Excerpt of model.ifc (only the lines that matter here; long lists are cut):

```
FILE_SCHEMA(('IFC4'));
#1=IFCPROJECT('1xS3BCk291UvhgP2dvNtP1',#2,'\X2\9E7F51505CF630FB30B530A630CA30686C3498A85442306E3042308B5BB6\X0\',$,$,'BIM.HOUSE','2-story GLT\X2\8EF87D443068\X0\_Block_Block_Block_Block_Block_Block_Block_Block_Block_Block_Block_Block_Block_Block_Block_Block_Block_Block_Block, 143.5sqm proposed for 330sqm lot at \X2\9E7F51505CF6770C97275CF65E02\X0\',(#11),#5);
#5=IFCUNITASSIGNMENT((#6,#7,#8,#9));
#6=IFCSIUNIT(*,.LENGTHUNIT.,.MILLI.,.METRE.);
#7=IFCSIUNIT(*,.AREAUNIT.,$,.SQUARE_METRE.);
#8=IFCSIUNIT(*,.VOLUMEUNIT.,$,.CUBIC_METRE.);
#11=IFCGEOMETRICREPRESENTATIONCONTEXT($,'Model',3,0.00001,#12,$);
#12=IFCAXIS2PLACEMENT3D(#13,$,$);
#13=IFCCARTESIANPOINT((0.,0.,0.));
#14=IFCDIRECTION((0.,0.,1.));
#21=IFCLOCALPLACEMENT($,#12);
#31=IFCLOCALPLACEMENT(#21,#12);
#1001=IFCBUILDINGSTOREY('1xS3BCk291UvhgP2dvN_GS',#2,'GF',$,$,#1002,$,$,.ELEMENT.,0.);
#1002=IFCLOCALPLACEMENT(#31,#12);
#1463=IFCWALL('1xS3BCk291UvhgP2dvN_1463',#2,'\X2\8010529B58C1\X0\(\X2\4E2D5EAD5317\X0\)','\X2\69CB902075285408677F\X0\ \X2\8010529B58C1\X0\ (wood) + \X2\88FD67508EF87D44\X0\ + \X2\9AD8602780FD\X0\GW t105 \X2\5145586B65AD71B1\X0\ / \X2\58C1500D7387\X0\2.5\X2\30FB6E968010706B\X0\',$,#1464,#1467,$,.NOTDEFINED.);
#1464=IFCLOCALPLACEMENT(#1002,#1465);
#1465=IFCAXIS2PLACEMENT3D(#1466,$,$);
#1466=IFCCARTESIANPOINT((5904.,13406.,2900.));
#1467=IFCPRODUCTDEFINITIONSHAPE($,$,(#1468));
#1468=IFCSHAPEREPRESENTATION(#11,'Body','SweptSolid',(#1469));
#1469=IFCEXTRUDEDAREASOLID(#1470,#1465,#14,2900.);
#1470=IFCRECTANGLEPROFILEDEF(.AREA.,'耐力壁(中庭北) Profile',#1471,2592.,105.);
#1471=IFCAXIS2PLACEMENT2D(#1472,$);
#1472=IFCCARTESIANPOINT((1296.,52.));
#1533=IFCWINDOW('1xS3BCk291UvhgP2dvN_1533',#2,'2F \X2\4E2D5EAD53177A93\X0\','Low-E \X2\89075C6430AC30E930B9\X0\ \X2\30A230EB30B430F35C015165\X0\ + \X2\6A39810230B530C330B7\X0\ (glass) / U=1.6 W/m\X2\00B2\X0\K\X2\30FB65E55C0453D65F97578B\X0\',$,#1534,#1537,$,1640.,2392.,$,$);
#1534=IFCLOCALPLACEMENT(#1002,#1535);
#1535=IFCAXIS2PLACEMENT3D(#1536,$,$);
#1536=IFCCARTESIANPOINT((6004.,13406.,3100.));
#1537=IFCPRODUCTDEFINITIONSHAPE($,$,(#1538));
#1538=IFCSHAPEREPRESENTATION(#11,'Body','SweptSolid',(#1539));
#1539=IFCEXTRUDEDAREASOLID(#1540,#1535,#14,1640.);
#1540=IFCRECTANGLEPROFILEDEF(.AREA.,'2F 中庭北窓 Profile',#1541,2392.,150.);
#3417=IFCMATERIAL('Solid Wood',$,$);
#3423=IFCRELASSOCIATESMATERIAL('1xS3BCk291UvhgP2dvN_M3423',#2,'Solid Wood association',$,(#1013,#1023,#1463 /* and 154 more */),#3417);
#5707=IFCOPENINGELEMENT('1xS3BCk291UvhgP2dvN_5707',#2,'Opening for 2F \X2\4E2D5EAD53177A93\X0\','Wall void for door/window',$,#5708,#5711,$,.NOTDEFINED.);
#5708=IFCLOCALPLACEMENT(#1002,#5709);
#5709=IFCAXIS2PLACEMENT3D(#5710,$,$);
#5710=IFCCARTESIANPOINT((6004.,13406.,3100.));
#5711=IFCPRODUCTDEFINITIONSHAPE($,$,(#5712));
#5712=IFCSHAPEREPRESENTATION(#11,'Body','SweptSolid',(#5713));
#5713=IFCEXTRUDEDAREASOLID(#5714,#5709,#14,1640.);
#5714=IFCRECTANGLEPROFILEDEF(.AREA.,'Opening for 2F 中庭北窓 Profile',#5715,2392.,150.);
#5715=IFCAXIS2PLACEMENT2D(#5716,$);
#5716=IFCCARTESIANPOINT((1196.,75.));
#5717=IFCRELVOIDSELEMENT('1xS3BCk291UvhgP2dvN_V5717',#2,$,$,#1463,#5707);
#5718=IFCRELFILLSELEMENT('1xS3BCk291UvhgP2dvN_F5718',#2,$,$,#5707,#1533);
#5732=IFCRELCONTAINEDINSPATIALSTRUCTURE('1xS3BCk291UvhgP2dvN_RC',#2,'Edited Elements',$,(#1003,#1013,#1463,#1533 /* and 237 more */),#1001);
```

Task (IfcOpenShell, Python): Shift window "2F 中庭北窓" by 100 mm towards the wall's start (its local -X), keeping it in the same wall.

```python
import ifcopenshell
import ifcopenshell.api.geometry
import ifcopenshell.util.placement
import ifcopenshell.util.unit

model = ifcopenshell.open("model.ifc")
unit_scale = ifcopenshell.util.unit.calculate_unit_scale(model)

window = model.by_id(1533)
opening = window.FillsVoids[0].RelatingOpeningElement
wall = opening.VoidsElements[0].RelatingBuildingElement

wall_matrix = ifcopenshell.util.placement.get_local_placement(wall.ObjectPlacement)
shift = wall_matrix[:3, 0] * -0.1 / unit_scale
before = ifcopenshell.util.placement.get_local_placement(window.ObjectPlacement)[:3, 3].copy()

# The window is not placed relative to its opening, so move both.
for product in (opening, window):
    matrix = ifcopenshell.util.placement.get_local_placement(product.ObjectPlacement)
    matrix[:3, 3] += shift
    ifcopenshell.api.geometry.edit_object_placement(model, product=product, matrix=matrix, is_si=False)

after = ifcopenshell.util.placement.get_local_placement(window.ObjectPlacement)[:3, 3]
print("window moved by", (after - before).round(3) + 0.0)

model.write("model-out.ifc")
```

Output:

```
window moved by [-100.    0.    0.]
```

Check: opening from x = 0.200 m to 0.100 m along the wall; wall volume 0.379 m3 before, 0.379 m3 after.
